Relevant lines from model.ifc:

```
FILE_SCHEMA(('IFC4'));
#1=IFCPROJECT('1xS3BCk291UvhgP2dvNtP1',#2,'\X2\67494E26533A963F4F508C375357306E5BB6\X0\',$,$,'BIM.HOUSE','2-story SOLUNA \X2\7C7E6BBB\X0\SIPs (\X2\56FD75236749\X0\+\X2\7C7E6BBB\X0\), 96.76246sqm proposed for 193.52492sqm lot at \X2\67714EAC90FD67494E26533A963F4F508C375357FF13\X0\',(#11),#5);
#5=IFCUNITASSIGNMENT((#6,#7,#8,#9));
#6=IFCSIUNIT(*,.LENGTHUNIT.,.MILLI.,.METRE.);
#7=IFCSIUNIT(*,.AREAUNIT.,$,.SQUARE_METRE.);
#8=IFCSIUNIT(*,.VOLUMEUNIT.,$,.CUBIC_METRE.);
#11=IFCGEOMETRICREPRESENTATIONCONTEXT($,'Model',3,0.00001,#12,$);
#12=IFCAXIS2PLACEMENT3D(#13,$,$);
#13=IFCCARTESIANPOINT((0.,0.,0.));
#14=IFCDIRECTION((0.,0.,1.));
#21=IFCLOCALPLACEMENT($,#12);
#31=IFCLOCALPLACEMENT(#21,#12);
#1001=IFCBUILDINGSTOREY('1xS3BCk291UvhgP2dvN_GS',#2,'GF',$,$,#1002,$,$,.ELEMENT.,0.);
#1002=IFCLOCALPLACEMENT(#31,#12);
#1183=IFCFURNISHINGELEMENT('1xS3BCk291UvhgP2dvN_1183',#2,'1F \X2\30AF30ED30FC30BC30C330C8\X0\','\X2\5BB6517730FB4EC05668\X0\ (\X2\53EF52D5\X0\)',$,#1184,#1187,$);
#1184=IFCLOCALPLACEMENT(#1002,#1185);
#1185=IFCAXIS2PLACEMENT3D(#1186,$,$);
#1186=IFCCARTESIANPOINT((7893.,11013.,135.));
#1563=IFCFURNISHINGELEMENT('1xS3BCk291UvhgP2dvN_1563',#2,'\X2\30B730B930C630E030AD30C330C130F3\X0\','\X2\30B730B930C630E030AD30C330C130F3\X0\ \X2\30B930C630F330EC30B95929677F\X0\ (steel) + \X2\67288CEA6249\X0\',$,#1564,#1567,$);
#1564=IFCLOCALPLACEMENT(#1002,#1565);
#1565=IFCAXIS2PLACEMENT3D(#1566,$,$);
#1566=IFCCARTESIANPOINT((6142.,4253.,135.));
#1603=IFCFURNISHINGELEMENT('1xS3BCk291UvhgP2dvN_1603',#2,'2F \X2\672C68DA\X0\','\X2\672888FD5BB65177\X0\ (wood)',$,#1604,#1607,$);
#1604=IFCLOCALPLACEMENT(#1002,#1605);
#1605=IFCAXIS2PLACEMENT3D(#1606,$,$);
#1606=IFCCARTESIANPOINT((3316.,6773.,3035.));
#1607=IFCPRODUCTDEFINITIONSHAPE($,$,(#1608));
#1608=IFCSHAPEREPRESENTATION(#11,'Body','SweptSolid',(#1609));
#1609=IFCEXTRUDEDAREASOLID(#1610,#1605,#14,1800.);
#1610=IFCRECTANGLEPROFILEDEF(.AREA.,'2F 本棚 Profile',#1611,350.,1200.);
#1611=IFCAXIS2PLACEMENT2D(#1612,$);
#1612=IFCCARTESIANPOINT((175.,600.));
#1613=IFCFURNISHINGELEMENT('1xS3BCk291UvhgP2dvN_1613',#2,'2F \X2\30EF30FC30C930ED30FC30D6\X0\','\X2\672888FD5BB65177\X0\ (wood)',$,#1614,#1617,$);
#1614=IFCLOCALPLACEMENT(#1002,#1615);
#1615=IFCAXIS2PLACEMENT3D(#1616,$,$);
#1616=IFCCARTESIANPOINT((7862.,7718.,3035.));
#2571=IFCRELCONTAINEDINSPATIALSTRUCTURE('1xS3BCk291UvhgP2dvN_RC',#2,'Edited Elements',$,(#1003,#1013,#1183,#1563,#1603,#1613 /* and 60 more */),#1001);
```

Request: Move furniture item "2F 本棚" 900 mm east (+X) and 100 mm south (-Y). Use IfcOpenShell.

```python
import ifcopenshell
import ifcopenshell.api.geometry
import ifcopenshell.util.placement

model = ifcopenshell.open("model.ifc")

item = model.by_guid("1xS3BCk291UvhgP2dvN_1603")
matrix = ifcopenshell.util.placement.get_local_placement(item.ObjectPlacement)
matrix[0, 3] += 900.0
matrix[1, 3] -= 100.0
ifcopenshell.api.geometry.edit_object_placement(model, product=item, matrix=matrix, is_si=False)

print(ifcopenshell.util.placement.get_local_placement(item.ObjectPlacement).round(3) + 0.0)

model.write("model_v2.ifc")
```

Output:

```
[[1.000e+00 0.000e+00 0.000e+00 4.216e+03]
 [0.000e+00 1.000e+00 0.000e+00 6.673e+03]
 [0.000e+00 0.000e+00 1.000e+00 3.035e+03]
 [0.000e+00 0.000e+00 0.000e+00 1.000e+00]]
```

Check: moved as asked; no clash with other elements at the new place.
